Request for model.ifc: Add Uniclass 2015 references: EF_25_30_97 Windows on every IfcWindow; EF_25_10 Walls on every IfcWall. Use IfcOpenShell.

First a look at what the model holds.

```python
import ifcopenshell

model = ifcopenshell.open("model.ifc")
print(model.schema)
print("classifications:", [c.Name for c in model.by_type("IfcClassification")])
for ifc_class in ("IfcDoor", "IfcRoof", "IfcStair", "IfcWall", "IfcWindow"):
    print(ifc_class, len(model.by_type(ifc_class)))
```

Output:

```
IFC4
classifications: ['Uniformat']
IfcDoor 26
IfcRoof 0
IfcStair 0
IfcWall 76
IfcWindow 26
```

```python
import ifcopenshell
import ifcopenshell.api.classification

model = ifcopenshell.open("model.ifc")

system = ifcopenshell.api.classification.add_classification(model, classification="Uniclass 2015")

codes = {
    "IfcWindow": ("EF_25_30_97", "Windows"),
    "IfcWall": ("EF_25_10", "Walls"),
}
for ifc_class, (code, name) in codes.items():
    products = model.by_type(ifc_class)
    ifcopenshell.api.classification.add_reference(
        model, products=products, classification=system, identification=code, name=name
    )
    print(code, len(products))

model.write("model-out.ifc")
```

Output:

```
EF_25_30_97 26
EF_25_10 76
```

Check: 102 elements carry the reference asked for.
